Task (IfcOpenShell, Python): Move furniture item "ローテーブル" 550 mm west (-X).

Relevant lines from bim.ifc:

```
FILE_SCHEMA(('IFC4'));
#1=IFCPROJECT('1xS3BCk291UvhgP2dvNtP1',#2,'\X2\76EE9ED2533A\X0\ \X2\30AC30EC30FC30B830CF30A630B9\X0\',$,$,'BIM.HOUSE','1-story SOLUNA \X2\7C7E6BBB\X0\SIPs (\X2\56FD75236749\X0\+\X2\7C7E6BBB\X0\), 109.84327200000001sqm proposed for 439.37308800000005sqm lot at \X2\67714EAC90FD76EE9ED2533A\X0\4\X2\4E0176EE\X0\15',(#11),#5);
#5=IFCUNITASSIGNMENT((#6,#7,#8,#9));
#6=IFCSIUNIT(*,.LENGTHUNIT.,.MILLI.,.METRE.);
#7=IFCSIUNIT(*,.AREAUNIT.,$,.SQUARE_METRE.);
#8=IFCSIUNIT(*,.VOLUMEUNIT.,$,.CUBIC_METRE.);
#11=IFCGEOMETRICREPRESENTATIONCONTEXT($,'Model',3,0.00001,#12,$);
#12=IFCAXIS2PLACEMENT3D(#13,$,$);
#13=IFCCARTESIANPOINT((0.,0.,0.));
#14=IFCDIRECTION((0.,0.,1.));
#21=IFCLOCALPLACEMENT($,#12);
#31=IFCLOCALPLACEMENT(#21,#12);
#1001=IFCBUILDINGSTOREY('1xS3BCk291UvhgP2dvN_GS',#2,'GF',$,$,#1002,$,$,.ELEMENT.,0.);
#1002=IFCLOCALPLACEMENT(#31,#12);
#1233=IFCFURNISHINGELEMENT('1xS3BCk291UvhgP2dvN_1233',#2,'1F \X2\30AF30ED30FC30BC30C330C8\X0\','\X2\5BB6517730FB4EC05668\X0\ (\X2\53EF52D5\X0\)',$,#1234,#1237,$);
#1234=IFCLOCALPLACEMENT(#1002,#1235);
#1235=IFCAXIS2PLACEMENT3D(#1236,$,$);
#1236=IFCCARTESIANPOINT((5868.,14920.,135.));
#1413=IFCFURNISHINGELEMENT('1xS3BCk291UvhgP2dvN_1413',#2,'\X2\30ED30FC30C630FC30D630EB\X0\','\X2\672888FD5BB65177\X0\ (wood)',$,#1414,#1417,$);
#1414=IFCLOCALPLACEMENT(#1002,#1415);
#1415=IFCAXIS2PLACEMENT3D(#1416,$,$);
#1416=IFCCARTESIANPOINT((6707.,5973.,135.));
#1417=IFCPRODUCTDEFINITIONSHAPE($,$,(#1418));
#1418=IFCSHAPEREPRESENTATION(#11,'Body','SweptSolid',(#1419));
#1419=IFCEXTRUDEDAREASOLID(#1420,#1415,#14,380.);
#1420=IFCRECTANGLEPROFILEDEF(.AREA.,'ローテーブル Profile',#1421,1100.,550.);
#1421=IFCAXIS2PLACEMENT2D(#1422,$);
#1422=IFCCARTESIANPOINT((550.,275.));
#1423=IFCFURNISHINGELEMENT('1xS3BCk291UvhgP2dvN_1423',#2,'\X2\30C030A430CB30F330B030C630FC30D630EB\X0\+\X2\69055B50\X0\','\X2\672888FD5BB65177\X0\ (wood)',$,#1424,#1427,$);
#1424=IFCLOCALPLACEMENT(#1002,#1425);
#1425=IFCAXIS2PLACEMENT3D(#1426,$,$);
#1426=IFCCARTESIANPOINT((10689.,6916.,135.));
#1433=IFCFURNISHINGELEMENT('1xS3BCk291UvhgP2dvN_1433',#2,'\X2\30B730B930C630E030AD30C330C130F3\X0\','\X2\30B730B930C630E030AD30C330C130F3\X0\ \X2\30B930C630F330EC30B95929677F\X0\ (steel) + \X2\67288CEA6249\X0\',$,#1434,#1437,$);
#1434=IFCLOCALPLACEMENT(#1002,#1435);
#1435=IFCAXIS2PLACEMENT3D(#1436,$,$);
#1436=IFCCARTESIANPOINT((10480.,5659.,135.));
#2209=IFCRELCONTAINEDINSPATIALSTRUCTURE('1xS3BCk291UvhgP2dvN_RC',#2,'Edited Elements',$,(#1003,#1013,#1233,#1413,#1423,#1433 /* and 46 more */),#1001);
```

```python
import ifcopenshell
import ifcopenshell.api.geometry
import ifcopenshell.util.placement
import ifcopenshell.util.unit

model = ifcopenshell.open("bim.ifc")
unit_scale = ifcopenshell.util.unit.calculate_unit_scale(model)

item = model.by_guid("1xS3BCk291UvhgP2dvN_1413")
matrix = ifcopenshell.util.placement.get_local_placement(item.ObjectPlacement)
matrix[0, 3] -= 0.55 / unit_scale
ifcopenshell.api.geometry.edit_object_placement(model, product=item, matrix=matrix, is_si=False)

print(ifcopenshell.util.placement.get_local_placement(item.ObjectPlacement).round(3) + 0.0)

model.write("bim-out.ifc")
```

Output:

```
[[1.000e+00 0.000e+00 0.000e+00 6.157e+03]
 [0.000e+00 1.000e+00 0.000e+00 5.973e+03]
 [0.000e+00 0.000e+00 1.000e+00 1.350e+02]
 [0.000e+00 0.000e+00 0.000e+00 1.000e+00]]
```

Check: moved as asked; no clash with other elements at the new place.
